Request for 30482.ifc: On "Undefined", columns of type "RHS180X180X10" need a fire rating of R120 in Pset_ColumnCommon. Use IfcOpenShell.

First a look at what the model holds.

```python
import ifcopenshell
import ifcopenshell.util.element

model = ifcopenshell.open("30482.ifc")
print(model.schema)
storey = next(s for s in model.by_type("IfcBuildingStorey") if s.Name == "Undefined")
columns = [e for e in ifcopenshell.util.element.get_decomposition(storey) if e.is_a("IfcColumn")]
seen = {}
for e in columns:
    element_type = ifcopenshell.util.element.get_type(e)
    key = (element_type.Name if element_type != e and element_type else None, ifcopenshell.util.element.get_pset(e, "Pset_ColumnCommon", "FireRating"))
    seen[key] = seen.get(key, 0) + 1
for (name, value), count in sorted(seen.items(), key=str):
    print(count, "x", name, "|", value)
```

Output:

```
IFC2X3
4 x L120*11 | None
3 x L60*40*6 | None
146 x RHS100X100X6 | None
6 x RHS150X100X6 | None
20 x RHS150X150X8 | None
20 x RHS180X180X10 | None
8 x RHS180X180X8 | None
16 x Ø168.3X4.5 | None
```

```python
import ifcopenshell
import ifcopenshell.api.pset
import ifcopenshell.util.element

model = ifcopenshell.open("30482.ifc")

storey = next(s for s in model.by_type("IfcBuildingStorey") if s.Name == "Undefined")
columns = [e for e in ifcopenshell.util.element.get_decomposition(storey) if e.is_a("IfcColumn")]

count = 0
for e in columns:
    element_type = ifcopenshell.util.element.get_type(e)
    if element_type in (None, e) or element_type.Name != "RHS180X180X10":
        continue
    found = ifcopenshell.util.element.get_pset(e, "Pset_ColumnCommon", should_inherit=False)
    if found:
        pset = model.by_id(found["id"])
        if len(ifcopenshell.util.element.get_elements_by_pset(pset)) > 1:
            pset = ifcopenshell.api.pset.unshare_pset(model, products=[e], pset=pset)[0]
    else:
        pset = ifcopenshell.api.pset.add_pset(model, product=e, name="Pset_ColumnCommon")
    ifcopenshell.api.pset.edit_pset(model, pset=pset, properties={"FireRating": "R120"})
    count += 1

print(count, "columns updated")

model.write("30482_edited.ifc")
```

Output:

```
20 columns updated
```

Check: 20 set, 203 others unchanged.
